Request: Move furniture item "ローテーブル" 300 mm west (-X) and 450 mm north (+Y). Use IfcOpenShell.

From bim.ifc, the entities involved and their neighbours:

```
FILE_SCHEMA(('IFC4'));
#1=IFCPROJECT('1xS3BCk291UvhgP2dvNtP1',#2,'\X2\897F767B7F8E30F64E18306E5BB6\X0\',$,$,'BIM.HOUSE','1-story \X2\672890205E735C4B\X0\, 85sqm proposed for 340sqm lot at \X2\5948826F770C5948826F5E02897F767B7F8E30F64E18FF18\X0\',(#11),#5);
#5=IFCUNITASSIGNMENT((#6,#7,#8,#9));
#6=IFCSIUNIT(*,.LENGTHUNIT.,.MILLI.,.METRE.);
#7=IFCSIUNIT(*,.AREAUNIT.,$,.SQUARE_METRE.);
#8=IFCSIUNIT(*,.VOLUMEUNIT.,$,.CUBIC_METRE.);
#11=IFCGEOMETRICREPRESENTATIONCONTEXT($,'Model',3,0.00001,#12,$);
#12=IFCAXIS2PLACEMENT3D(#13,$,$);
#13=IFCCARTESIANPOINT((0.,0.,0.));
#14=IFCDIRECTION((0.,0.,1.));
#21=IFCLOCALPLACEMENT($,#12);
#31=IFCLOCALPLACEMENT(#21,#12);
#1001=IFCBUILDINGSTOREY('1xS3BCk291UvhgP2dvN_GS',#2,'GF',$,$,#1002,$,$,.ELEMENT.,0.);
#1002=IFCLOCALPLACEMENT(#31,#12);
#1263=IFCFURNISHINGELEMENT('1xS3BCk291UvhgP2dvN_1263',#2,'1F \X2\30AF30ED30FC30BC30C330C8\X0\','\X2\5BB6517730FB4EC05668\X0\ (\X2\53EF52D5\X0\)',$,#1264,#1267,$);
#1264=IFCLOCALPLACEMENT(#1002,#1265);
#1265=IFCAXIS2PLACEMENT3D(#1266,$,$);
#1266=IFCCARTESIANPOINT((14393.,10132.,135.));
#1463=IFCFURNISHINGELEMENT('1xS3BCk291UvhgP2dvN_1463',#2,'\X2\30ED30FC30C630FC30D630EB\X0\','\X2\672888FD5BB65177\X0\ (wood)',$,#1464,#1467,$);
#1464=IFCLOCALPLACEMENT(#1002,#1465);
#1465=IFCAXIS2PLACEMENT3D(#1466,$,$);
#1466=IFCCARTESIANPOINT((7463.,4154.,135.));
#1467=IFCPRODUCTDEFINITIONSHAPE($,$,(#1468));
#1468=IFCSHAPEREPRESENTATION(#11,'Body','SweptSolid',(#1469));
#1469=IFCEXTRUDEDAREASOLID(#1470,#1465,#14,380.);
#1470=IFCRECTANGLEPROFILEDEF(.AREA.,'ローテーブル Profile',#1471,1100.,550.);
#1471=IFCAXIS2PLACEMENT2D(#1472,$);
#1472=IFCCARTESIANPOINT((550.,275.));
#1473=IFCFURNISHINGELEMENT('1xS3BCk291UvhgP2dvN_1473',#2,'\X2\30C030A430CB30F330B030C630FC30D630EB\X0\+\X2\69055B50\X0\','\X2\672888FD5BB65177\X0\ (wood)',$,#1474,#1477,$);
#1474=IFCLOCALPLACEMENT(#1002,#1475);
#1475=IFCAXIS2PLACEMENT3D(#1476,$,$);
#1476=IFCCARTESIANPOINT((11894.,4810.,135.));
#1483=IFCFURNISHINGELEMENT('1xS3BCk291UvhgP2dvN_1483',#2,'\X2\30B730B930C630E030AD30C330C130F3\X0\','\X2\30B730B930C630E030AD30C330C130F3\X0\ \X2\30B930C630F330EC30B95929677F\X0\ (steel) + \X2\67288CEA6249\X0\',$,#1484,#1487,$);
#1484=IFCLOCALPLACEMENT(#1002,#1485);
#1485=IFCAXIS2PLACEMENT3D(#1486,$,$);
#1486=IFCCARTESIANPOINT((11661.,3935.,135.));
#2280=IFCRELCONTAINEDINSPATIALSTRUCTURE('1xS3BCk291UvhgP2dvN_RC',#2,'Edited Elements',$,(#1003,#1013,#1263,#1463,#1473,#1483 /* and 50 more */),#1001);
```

```python
import ifcopenshell
import ifcopenshell.api.geometry
import ifcopenshell.util.placement
import ifcopenshell.util.unit

model = ifcopenshell.open("bim.ifc")
unit_scale = ifcopenshell.util.unit.calculate_unit_scale(model)

item = model.by_guid("1xS3BCk291UvhgP2dvN_1463")
matrix = ifcopenshell.util.placement.get_local_placement(item.ObjectPlacement)
matrix[0, 3] -= 0.3 / unit_scale
matrix[1, 3] += 0.45 / unit_scale
ifcopenshell.api.geometry.edit_object_placement(model, product=item, matrix=matrix, is_si=False)

print(ifcopenshell.util.placement.get_local_placement(item.ObjectPlacement).round(3) + 0.0)

model.write("bim_rev.ifc")
```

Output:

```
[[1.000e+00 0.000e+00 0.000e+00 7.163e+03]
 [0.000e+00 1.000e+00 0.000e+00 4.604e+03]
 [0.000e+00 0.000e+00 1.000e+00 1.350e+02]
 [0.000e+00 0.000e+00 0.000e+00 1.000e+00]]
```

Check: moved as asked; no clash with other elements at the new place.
